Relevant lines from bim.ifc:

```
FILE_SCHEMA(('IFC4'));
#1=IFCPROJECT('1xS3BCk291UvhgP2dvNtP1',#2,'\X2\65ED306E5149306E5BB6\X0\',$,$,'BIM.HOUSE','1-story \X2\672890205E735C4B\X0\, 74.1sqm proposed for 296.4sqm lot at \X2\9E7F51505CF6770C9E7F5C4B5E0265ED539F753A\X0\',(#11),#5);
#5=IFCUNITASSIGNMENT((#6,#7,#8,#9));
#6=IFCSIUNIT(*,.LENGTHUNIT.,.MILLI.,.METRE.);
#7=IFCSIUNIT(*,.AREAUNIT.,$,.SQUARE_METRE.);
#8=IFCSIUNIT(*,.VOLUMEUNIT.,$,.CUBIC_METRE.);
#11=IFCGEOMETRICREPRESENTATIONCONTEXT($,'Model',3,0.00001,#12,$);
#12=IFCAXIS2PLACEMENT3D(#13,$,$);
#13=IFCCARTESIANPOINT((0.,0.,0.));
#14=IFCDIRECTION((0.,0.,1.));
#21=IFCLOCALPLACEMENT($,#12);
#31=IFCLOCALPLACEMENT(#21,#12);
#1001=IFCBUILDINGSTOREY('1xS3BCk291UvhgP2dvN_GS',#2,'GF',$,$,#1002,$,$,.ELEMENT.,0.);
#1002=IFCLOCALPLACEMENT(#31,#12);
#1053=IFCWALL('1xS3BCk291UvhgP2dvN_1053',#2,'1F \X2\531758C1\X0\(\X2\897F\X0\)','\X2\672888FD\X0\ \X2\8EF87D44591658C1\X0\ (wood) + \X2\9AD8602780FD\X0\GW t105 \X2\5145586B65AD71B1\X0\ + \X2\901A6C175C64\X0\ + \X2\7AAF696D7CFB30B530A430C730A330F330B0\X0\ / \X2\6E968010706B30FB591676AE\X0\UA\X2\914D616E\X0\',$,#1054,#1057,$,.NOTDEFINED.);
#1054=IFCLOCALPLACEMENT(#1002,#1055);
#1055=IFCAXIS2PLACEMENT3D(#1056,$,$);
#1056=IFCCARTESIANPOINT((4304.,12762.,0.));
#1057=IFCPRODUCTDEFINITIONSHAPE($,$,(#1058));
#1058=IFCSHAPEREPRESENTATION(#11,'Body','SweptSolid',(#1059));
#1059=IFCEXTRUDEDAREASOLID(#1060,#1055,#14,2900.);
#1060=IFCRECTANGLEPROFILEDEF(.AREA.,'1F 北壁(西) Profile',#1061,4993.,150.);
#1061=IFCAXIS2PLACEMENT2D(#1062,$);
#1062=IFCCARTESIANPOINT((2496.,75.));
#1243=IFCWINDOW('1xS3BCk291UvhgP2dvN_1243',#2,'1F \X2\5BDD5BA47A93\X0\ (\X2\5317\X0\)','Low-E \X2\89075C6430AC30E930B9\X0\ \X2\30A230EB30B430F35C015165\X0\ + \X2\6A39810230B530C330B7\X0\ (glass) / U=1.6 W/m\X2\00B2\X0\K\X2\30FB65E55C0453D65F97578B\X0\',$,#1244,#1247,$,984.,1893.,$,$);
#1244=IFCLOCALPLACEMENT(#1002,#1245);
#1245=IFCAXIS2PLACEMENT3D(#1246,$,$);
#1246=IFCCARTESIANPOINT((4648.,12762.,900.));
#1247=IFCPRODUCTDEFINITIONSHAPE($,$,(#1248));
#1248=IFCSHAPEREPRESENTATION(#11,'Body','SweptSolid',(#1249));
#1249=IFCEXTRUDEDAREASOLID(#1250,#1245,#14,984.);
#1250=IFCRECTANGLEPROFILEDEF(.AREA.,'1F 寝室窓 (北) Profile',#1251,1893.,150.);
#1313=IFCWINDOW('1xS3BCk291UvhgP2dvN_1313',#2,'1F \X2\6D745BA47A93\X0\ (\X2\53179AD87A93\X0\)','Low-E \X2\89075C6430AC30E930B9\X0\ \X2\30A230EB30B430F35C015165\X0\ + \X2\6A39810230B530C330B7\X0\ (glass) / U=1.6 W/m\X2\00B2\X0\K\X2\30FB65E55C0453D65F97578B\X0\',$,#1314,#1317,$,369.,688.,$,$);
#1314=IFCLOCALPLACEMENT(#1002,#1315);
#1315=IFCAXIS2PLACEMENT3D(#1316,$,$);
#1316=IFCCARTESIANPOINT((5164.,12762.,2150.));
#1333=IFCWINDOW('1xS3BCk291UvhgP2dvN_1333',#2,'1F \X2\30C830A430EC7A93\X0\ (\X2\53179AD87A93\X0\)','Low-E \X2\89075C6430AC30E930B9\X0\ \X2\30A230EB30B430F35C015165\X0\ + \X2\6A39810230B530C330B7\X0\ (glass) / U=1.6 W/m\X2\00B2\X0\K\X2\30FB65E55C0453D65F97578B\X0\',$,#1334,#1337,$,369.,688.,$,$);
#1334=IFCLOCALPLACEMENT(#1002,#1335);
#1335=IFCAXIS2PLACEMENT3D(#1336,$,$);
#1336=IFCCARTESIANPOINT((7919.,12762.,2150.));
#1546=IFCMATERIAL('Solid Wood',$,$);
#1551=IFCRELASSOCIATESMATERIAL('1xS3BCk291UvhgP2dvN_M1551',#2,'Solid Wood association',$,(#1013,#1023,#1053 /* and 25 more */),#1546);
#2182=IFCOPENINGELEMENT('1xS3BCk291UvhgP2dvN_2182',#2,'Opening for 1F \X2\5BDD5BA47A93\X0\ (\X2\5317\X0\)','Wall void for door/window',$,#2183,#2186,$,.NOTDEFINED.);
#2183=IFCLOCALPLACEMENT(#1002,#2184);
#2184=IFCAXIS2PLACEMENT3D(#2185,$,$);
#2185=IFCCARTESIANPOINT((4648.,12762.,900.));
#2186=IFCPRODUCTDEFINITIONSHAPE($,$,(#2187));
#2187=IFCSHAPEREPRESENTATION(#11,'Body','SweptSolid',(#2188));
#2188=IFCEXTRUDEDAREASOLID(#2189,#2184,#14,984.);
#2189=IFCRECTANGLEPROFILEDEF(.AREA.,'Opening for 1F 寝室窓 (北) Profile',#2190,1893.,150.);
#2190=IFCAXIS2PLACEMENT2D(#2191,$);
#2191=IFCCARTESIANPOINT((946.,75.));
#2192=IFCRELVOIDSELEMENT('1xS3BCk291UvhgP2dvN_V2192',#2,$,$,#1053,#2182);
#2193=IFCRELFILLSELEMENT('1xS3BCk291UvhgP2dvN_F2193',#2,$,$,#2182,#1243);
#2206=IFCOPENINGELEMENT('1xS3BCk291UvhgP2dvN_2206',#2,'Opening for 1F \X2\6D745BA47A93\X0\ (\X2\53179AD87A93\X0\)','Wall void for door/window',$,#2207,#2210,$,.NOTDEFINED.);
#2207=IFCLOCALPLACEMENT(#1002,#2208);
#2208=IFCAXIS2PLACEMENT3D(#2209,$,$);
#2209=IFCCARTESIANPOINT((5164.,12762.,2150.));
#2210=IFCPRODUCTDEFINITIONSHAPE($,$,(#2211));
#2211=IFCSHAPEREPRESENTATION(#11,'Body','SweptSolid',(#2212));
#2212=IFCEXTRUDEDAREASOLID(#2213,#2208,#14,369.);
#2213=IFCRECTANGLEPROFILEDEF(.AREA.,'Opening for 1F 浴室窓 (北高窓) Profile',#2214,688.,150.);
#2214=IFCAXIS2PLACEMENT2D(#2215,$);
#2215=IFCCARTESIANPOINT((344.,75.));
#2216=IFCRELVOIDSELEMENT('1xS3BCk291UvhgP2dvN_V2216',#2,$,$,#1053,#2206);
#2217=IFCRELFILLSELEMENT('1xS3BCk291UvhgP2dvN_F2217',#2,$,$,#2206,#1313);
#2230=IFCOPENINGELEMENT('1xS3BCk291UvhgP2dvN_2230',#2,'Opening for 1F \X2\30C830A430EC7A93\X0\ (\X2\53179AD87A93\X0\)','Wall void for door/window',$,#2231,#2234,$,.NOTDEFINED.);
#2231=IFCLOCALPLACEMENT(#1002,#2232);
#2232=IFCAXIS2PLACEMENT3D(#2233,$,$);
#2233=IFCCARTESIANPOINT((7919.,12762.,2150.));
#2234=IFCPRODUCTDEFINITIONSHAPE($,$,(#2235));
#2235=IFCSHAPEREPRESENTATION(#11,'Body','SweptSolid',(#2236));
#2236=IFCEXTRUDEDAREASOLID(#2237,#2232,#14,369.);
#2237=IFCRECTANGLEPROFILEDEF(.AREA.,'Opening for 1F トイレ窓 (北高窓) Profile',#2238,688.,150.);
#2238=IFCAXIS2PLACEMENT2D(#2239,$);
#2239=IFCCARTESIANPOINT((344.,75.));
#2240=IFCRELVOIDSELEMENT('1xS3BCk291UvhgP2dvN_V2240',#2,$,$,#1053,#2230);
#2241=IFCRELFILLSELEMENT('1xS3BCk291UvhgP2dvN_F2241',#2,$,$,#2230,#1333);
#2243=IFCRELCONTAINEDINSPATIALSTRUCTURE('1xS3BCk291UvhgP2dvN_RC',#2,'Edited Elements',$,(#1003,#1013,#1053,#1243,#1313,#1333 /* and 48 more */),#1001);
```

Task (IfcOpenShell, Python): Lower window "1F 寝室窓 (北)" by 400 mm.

```python
import numpy as np
import ifcopenshell
import ifcopenshell.api.geometry
import ifcopenshell.util.placement
import ifcopenshell.util.unit

model = ifcopenshell.open("bim.ifc")
unit_scale = ifcopenshell.util.unit.calculate_unit_scale(model)

window = model.by_id(1243)
opening = window.FillsVoids[0].RelatingOpeningElement
dz = -0.4 / unit_scale

shift = np.array([0.0, 0.0, dz])
# The window is not placed relative to its opening, so move both.
for product in (opening, window):
    matrix = ifcopenshell.util.placement.get_local_placement(product.ObjectPlacement)
    matrix[:3, 3] += shift
    ifcopenshell.api.geometry.edit_object_placement(model, product=product, matrix=matrix, is_si=False)

print(f"moved by {dz * unit_scale:+.3f} m")

model.write("bim_edited.ifc")
```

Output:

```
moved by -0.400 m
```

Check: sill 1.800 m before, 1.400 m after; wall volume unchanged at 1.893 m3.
